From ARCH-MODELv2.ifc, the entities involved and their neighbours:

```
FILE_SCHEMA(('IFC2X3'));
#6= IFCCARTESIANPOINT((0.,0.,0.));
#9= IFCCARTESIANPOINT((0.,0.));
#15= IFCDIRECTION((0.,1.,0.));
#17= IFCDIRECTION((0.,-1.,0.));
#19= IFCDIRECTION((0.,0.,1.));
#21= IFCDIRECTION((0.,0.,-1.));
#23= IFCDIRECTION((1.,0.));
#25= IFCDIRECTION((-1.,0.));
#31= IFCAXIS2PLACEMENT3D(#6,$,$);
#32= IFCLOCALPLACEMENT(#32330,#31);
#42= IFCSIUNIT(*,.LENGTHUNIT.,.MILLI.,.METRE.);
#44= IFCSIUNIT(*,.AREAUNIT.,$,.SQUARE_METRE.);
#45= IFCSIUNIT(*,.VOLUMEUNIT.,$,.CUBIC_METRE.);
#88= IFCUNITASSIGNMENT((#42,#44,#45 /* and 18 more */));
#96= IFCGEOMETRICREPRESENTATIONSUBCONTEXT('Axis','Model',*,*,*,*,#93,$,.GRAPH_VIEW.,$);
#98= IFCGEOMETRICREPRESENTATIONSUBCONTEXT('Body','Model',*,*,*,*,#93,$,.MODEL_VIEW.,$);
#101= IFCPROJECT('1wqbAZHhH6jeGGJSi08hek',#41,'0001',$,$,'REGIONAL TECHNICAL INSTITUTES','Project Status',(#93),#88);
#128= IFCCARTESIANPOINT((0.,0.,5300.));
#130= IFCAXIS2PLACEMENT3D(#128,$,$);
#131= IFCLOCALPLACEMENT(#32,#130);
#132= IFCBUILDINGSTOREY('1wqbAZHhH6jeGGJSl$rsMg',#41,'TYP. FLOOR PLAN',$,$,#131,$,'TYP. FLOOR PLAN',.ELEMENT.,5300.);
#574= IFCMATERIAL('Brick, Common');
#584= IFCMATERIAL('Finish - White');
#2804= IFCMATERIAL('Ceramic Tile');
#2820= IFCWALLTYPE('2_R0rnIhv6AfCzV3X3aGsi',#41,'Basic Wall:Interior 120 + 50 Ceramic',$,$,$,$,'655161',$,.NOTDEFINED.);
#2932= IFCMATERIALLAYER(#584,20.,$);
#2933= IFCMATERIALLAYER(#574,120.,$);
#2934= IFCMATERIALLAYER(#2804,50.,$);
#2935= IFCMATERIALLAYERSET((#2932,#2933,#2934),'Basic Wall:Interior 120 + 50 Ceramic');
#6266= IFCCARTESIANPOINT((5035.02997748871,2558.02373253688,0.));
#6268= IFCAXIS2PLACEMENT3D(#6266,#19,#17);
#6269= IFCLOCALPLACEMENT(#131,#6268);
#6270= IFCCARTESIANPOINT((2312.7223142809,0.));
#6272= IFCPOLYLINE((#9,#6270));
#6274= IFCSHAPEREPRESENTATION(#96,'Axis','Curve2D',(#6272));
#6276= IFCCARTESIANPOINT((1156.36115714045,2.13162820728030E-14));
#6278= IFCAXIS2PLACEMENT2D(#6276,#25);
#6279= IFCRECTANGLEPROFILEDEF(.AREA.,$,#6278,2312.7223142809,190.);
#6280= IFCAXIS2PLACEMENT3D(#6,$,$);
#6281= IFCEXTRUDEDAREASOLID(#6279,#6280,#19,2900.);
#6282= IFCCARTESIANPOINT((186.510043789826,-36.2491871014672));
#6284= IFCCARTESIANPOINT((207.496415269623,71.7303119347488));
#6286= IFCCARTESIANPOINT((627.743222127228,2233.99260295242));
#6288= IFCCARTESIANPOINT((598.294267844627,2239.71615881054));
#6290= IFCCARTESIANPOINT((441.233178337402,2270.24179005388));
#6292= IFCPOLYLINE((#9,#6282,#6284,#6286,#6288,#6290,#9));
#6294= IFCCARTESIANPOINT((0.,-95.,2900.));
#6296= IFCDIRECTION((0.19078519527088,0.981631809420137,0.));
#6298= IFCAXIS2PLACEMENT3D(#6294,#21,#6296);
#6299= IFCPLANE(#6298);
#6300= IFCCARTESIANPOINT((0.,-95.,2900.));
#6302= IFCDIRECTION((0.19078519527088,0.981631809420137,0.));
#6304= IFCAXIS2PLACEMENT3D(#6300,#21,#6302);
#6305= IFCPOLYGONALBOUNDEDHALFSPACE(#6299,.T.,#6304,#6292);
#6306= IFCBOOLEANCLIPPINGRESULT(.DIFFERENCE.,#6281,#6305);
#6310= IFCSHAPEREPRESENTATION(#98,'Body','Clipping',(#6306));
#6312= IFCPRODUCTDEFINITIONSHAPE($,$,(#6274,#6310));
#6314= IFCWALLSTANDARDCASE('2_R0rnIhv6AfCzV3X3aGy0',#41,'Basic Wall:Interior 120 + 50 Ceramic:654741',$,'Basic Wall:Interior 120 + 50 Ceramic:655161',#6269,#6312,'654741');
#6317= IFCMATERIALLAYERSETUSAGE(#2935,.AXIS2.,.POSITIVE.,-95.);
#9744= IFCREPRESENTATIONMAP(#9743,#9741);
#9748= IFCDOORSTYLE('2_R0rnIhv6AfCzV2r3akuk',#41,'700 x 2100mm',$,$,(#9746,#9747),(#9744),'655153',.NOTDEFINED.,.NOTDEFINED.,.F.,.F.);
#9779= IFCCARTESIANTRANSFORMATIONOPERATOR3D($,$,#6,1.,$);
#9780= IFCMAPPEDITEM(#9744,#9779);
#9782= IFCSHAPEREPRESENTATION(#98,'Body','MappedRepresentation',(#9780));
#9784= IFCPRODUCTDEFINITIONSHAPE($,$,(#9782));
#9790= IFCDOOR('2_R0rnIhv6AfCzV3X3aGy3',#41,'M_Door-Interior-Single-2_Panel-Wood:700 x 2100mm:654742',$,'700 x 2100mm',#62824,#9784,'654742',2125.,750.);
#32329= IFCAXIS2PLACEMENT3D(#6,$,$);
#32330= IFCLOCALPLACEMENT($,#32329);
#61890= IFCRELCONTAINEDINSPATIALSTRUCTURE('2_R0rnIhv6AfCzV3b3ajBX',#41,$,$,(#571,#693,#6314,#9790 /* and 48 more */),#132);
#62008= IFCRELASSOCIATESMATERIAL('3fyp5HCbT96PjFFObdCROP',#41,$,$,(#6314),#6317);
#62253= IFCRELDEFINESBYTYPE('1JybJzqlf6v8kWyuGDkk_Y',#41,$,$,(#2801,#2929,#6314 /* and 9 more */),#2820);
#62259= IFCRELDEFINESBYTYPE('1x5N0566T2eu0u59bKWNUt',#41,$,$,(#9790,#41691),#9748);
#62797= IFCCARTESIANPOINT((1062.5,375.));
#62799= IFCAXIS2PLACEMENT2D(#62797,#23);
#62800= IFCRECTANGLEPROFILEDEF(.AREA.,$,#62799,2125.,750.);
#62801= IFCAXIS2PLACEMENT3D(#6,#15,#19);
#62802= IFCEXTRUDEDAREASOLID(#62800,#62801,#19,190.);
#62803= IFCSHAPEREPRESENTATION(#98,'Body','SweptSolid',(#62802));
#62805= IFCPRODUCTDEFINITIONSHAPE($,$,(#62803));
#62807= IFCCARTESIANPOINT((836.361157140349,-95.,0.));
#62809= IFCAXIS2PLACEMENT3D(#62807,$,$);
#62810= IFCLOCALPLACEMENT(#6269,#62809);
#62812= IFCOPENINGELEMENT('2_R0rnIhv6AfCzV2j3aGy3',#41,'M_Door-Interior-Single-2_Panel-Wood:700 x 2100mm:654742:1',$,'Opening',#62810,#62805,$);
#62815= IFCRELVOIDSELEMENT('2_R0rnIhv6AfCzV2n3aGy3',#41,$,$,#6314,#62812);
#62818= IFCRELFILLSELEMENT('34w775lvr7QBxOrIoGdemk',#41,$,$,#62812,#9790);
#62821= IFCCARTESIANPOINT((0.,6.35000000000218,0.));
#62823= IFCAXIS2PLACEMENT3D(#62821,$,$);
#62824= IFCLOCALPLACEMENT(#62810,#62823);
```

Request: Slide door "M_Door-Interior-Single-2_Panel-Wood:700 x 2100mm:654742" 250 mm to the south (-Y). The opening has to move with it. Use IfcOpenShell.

```python
import ifcopenshell
import ifcopenshell.api.geometry
import ifcopenshell.util.placement
import ifcopenshell.util.unit

model = ifcopenshell.open("ARCH-MODELv2.ifc")
unit_scale = ifcopenshell.util.unit.calculate_unit_scale(model)

door = model.by_guid("2_R0rnIhv6AfCzV3X3aGy3")
opening = door.FillsVoids[0].RelatingOpeningElement
wall = opening.VoidsElements[0].RelatingBuildingElement

wall_matrix = ifcopenshell.util.placement.get_local_placement(wall.ObjectPlacement)
shift = wall_matrix[:3, 0] * 0.25 / unit_scale
before = ifcopenshell.util.placement.get_local_placement(door.ObjectPlacement)[:3, 3].copy()

# The door is placed relative to its opening, so it follows when the opening moves.
matrix = ifcopenshell.util.placement.get_local_placement(opening.ObjectPlacement)
matrix[:3, 3] += shift
ifcopenshell.api.geometry.edit_object_placement(
    model, product=opening, matrix=matrix, is_si=False, should_transform_children=True
)

after = ifcopenshell.util.placement.get_local_placement(door.ObjectPlacement)[:3, 3]
print("door moved by", (after - before).round(3) + 0.0)

model.write("ARCH-MODELv2_edited.ifc")
```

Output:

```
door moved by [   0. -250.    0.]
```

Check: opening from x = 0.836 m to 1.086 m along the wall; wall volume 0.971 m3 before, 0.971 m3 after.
